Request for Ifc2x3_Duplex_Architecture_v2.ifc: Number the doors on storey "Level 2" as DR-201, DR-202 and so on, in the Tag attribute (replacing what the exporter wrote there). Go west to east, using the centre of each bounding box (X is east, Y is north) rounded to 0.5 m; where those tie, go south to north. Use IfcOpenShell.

First a look at what the model holds.

```python
import ifcopenshell
import ifcopenshell.util.element
import ifcopenshell.util.placement

model = ifcopenshell.open("Ifc2x3_Duplex_Architecture_v2.ifc")
print(model.schema)
storey = next(s for s in model.by_type("IfcBuildingStorey") if s.Name == "Level 2")
doors = [e for e in ifcopenshell.util.element.get_decomposition(storey) if e.is_a("IfcDoor")]
for e in sorted(doors, key=lambda e: e.id()):
    origin = ifcopenshell.util.placement.get_local_placement(e.ObjectPlacement)[:3, 3]
    print(e.id(), e.Tag, e.Name, origin.round(2) + 0.0, sep=" | ")
```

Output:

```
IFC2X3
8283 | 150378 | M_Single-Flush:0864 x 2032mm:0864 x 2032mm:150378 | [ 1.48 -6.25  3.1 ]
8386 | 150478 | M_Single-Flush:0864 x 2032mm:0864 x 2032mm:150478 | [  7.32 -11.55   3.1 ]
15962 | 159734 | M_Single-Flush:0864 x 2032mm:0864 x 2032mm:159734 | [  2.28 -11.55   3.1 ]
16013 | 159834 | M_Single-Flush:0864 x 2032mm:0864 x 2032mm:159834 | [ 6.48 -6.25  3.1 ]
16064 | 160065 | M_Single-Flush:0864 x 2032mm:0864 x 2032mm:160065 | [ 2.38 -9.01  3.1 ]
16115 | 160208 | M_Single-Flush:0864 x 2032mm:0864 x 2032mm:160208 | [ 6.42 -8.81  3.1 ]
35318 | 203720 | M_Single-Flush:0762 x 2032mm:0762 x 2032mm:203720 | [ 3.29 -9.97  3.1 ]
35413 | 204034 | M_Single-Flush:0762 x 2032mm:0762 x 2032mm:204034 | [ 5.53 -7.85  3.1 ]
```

```python
import ifcopenshell
import ifcopenshell.geom
import ifcopenshell.util.element
import ifcopenshell.util.shape

model = ifcopenshell.open("Ifc2x3_Duplex_Architecture_v2.ifc")
settings = ifcopenshell.geom.settings()
settings.set("use-world-coords", True)


def centre(element):
    shape = ifcopenshell.geom.create_shape(settings, element)
    return ifcopenshell.util.shape.get_bbox_centroid(shape.geometry)


storey = next(s for s in model.by_type("IfcBuildingStorey") if s.Name == "Level 2")
doors = [e for e in ifcopenshell.util.element.get_decomposition(storey) if e.is_a("IfcDoor")]

# Insertion points can sit at a corner or the storey origin, so sort by the geometry (in metres).
centres = {e: centre(e) for e in doors}
doors.sort(key=lambda e: (round(centres[e][0] / 0.5), centres[e][1]))

for i, e in enumerate(doors, start=1):
    number = f"DR-2{i:02d}"
    e.Tag = number
    print(e.id(), number)

model.write("Ifc2x3_Duplex_Architecture_v2_v2.ifc")
```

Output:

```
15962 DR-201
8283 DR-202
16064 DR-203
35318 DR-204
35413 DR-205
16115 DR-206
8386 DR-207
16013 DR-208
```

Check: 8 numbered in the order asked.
